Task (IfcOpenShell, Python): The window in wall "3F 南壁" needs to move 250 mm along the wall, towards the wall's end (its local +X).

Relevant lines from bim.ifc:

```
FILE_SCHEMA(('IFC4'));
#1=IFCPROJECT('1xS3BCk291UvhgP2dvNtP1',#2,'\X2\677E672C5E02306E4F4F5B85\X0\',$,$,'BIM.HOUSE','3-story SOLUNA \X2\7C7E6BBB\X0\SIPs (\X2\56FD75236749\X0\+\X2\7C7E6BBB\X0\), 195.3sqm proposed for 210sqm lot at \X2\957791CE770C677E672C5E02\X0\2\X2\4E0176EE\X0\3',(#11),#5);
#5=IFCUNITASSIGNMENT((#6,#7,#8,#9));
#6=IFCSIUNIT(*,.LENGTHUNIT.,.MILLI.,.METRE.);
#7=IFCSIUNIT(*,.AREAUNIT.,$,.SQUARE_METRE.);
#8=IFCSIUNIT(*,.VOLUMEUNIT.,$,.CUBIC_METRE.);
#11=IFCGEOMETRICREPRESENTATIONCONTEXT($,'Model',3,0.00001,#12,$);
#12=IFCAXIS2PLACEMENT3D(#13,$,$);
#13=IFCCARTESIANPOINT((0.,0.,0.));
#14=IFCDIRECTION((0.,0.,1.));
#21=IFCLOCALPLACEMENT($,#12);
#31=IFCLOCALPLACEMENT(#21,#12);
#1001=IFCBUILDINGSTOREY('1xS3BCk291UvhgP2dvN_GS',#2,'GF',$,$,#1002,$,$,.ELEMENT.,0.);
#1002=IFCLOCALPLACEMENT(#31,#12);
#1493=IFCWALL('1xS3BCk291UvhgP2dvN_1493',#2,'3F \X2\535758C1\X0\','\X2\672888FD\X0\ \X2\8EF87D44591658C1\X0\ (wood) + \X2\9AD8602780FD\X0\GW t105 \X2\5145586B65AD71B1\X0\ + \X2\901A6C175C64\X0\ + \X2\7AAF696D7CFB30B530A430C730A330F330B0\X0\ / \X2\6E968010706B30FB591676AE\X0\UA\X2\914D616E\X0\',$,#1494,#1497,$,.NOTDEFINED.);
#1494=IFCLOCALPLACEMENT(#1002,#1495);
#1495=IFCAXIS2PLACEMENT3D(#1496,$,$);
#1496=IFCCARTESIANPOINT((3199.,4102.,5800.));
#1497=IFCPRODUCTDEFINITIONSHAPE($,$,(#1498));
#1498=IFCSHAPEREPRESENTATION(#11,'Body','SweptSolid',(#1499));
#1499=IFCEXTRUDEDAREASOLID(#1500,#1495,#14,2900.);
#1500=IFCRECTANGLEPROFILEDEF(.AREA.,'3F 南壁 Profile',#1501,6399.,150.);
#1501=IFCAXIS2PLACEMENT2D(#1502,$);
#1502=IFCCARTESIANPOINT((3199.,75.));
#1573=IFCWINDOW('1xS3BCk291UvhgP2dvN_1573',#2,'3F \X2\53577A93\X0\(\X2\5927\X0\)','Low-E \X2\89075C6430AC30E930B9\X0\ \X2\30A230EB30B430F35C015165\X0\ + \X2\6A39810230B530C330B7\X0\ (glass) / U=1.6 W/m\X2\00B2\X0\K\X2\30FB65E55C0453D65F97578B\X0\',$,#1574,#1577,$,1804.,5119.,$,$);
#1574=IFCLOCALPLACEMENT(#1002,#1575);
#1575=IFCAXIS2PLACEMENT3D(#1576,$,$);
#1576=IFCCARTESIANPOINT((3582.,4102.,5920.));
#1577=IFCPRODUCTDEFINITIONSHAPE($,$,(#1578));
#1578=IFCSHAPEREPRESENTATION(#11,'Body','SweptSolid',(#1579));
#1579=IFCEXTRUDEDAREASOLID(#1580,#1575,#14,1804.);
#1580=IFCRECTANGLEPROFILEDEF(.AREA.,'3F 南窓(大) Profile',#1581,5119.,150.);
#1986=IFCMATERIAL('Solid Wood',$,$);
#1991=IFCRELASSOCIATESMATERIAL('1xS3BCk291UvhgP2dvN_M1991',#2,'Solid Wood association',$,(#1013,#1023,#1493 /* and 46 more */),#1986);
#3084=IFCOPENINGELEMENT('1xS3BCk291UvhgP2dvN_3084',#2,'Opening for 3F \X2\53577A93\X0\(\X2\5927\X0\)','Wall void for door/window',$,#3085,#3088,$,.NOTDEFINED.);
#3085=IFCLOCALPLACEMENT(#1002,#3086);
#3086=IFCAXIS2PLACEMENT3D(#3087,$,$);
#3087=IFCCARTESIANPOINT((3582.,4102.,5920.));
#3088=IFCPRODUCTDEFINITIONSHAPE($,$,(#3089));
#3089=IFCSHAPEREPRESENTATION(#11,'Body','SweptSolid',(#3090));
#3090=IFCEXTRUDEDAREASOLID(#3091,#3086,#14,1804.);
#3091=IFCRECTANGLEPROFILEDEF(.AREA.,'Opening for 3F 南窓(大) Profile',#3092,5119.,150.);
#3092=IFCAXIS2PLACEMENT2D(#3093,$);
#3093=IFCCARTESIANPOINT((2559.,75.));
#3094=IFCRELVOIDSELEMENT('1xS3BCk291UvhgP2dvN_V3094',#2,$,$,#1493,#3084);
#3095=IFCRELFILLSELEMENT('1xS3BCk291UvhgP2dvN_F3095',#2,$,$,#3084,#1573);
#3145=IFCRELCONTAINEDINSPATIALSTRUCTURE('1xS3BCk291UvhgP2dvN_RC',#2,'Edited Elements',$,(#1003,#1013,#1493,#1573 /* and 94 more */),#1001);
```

```python
import ifcopenshell
import ifcopenshell.api.geometry
import ifcopenshell.util.placement
import ifcopenshell.util.unit

model = ifcopenshell.open("bim.ifc")
unit_scale = ifcopenshell.util.unit.calculate_unit_scale(model)

window = model.by_id(1573)
opening = window.FillsVoids[0].RelatingOpeningElement
wall = opening.VoidsElements[0].RelatingBuildingElement

wall_matrix = ifcopenshell.util.placement.get_local_placement(wall.ObjectPlacement)
shift = wall_matrix[:3, 0] * 0.25 / unit_scale
before = ifcopenshell.util.placement.get_local_placement(window.ObjectPlacement)[:3, 3].copy()

# The window is not placed relative to its opening, so move both.
for product in (opening, window):
    matrix = ifcopenshell.util.placement.get_local_placement(product.ObjectPlacement)
    matrix[:3, 3] += shift
    ifcopenshell.api.geometry.edit_object_placement(model, product=product, matrix=matrix, is_si=False)

after = ifcopenshell.util.placement.get_local_placement(window.ObjectPlacement)[:3, 3]
print("window moved by", (after - before).round(3) + 0.0)

model.write("bim_rev.ifc")
```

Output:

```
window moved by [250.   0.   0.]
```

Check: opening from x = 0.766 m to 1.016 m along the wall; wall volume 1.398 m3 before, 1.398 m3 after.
